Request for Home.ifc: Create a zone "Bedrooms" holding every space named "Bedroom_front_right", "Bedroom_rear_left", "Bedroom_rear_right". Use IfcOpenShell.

First a look at what the model holds.

```python
import ifcopenshell

model = ifcopenshell.open("Home.ifc")
print(model.schema)
seen = {}
for space in model.by_type("IfcSpace"):
    seen[space.LongName] = seen.get(space.LongName, 0) + 1
for name, count in sorted(seen.items(), key=str):
    print(count, "x", name)
print("zones:", [z.Name for z in model.by_type("IfcZone")][:20])
```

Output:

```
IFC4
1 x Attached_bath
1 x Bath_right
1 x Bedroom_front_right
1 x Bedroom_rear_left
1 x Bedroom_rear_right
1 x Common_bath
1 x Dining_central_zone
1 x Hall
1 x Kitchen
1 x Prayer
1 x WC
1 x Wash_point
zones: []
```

```python
import ifcopenshell
import ifcopenshell.api.group
import ifcopenshell.api.root

model = ifcopenshell.open("Home.ifc")

names = {"Bedroom_front_right", "Bedroom_rear_left", "Bedroom_rear_right"}
spaces = [s for s in model.by_type("IfcSpace") if s.LongName in names]

zone = ifcopenshell.api.root.create_entity(model, ifc_class="IfcZone", name="Bedrooms")
ifcopenshell.api.group.assign_group(model, products=spaces, group=zone)
print(len(spaces), "spaces in", zone.Name)

model.write("Home-out.ifc")
```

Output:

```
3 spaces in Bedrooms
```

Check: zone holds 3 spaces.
